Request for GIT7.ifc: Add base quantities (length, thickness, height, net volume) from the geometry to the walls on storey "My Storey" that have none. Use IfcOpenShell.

First a look at what the model holds.

```python
import ifcopenshell
import ifcopenshell.util.element
import ifcopenshell.util.unit

model = ifcopenshell.open("GIT7.ifc")
print(model.schema)
for unit_type in ("LENGTHUNIT", "AREAUNIT", "VOLUMEUNIT"):
    print(unit_type, ifcopenshell.util.unit.calculate_unit_scale(model, unit_type))
storey = next(s for s in model.by_type("IfcBuildingStorey") if s.Name == "My Storey")
walls = [e for e in ifcopenshell.util.element.get_decomposition(storey) if e.is_a("IfcWall")]
for e in sorted(walls, key=lambda e: e.id()):
    print(e.id(), e.is_a(), e.Name, list(ifcopenshell.util.element.get_psets(e, qtos_only=True)), sep=" | ")
```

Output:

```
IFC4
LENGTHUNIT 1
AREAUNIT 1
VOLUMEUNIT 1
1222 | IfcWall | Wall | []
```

```python
import ifcopenshell
import ifcopenshell.api.pset
import ifcopenshell.geom
import ifcopenshell.util.element
import ifcopenshell.util.shape
import ifcopenshell.util.unit

model = ifcopenshell.open("GIT7.ifc")
unit_scale = ifcopenshell.util.unit.calculate_unit_scale(model)
volume_scale = ifcopenshell.util.unit.calculate_unit_scale(model, "VOLUMEUNIT")
settings = ifcopenshell.geom.settings()

storey = next(s for s in model.by_type("IfcBuildingStorey") if s.Name == "My Storey")
walls = [e for e in ifcopenshell.util.element.get_decomposition(storey) if e.is_a("IfcWall")]

for e in sorted(walls, key=lambda e: e.id()):
    if ifcopenshell.util.element.get_psets(e, qtos_only=True, should_inherit=False):
        continue
    # Geometry comes back in metres, in the element's own axes.
    shape = ifcopenshell.geom.create_shape(settings, e)
    values = {
        "Length": ifcopenshell.util.shape.get_x(shape.geometry) / unit_scale,
        "Width": ifcopenshell.util.shape.get_y(shape.geometry) / unit_scale,
        "Height": ifcopenshell.util.shape.get_z(shape.geometry) / unit_scale,
        "NetVolume": ifcopenshell.util.shape.get_volume(shape.geometry) / volume_scale,
    }
    qto = ifcopenshell.api.pset.add_qto(model, product=e, name="Qto_WallBaseQuantities")
    ifcopenshell.api.pset.edit_qto(model, qto=qto, properties=values)
    print(e.id(), {k: round(v, 3) for k, v in values.items()})

model.write("GIT7_updated.ifc")
```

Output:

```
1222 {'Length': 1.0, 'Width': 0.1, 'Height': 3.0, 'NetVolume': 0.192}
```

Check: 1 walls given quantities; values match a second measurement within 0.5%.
